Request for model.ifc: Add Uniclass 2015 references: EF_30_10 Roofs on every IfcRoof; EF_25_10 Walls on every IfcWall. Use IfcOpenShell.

First a look at what the model holds.

```python
import ifcopenshell

model = ifcopenshell.open("model.ifc")
print(model.schema)
print("classifications:", [c.Name for c in model.by_type("IfcClassification")])
for ifc_class in ("IfcDoor", "IfcRoof", "IfcStair", "IfcWall", "IfcWindow"):
    print(ifc_class, len(model.by_type(ifc_class)))
```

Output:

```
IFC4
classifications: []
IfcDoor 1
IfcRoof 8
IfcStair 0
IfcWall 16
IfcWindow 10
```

```python
import ifcopenshell
import ifcopenshell.api.classification

model = ifcopenshell.open("model.ifc")

system = ifcopenshell.api.classification.add_classification(model, classification="Uniclass 2015")

codes = {
    "IfcRoof": ("EF_30_10", "Roofs"),
    "IfcWall": ("EF_25_10", "Walls"),
}
for ifc_class, (code, name) in codes.items():
    products = model.by_type(ifc_class)
    ifcopenshell.api.classification.add_reference(
        model, products=products, classification=system, identification=code, name=name
    )
    print(code, len(products))

model.write("model_rev.ifc")
```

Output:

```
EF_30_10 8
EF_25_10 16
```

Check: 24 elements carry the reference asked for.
